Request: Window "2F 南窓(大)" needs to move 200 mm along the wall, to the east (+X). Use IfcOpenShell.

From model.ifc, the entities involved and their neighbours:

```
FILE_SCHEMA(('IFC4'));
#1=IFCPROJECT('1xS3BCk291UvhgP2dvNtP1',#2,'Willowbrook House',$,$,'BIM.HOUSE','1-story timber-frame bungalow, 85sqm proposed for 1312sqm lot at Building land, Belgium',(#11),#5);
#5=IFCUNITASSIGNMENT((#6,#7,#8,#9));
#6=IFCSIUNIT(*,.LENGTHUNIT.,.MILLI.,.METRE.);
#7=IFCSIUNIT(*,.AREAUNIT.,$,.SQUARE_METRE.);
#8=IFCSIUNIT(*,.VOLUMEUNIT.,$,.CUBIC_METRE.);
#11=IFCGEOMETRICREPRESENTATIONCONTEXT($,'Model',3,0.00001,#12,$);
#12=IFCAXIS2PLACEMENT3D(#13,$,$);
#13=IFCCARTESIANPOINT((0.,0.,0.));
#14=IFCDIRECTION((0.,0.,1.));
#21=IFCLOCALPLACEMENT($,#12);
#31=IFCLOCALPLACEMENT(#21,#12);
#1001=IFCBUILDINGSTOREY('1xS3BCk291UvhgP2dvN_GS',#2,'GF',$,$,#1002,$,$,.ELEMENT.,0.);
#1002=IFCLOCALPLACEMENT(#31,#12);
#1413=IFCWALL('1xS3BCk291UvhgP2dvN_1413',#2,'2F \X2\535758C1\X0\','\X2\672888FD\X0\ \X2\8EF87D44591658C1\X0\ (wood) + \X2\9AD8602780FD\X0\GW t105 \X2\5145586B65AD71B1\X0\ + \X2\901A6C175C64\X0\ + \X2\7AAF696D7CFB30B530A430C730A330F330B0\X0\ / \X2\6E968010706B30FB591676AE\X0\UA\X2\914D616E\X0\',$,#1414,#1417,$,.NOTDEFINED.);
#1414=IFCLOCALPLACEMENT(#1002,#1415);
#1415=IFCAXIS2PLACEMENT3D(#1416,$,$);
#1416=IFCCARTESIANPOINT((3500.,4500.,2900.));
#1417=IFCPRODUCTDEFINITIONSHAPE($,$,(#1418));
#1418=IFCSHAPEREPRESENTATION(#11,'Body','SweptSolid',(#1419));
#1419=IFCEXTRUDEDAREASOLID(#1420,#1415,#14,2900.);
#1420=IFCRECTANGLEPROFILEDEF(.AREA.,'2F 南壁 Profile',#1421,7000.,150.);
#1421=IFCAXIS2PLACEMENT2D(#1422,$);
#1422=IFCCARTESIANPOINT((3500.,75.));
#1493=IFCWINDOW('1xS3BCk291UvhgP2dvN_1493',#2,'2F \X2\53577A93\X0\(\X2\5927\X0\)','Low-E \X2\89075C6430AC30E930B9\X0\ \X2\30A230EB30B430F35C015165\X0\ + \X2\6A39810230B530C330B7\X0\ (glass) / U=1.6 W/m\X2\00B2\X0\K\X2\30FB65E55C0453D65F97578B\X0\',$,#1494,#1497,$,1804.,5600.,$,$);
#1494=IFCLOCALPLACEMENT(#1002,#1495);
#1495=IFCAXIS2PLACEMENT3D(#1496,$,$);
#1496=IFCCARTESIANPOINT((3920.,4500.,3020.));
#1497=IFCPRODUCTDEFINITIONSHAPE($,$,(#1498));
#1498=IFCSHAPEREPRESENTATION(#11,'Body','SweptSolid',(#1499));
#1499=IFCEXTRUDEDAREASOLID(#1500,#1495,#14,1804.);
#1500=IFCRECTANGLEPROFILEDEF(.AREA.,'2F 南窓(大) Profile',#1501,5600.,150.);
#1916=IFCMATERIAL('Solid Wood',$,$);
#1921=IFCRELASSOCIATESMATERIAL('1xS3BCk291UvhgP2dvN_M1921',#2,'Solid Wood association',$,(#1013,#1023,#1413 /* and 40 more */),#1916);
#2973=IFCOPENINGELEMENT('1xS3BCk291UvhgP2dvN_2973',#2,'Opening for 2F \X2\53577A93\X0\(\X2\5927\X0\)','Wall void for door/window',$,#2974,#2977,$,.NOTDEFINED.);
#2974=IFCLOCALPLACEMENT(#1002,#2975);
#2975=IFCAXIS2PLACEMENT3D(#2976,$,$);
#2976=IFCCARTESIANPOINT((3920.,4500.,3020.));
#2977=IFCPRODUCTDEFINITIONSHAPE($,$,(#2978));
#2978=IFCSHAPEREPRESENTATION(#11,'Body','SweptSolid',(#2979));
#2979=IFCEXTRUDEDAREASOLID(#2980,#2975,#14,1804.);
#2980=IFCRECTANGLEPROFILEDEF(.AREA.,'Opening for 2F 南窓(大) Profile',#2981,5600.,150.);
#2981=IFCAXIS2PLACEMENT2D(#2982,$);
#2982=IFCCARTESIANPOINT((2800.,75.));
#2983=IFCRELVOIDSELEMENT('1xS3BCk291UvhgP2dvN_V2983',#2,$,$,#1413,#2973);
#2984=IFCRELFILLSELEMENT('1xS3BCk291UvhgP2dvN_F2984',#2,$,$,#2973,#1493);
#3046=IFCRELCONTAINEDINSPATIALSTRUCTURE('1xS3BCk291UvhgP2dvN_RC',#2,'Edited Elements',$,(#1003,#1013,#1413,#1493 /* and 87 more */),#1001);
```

```python
import ifcopenshell
import ifcopenshell.api.geometry
import ifcopenshell.util.placement
import ifcopenshell.util.unit

model = ifcopenshell.open("model.ifc")
unit_scale = ifcopenshell.util.unit.calculate_unit_scale(model)

window = model.by_id(1493)
opening = window.FillsVoids[0].RelatingOpeningElement
wall = opening.VoidsElements[0].RelatingBuildingElement

wall_matrix = ifcopenshell.util.placement.get_local_placement(wall.ObjectPlacement)
shift = wall_matrix[:3, 0] * 0.2 / unit_scale
before = ifcopenshell.util.placement.get_local_placement(window.ObjectPlacement)[:3, 3].copy()

# The window is not placed relative to its opening, so move both.
for product in (opening, window):
    matrix = ifcopenshell.util.placement.get_local_placement(product.ObjectPlacement)
    matrix[:3, 3] += shift
    ifcopenshell.api.geometry.edit_object_placement(model, product=product, matrix=matrix, is_si=False)

after = ifcopenshell.util.placement.get_local_placement(window.ObjectPlacement)[:3, 3]
print("window moved by", (after - before).round(3) + 0.0)

model.write("model_v2.ifc")
```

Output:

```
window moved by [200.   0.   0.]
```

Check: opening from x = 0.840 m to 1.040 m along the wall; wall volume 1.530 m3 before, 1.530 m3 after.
